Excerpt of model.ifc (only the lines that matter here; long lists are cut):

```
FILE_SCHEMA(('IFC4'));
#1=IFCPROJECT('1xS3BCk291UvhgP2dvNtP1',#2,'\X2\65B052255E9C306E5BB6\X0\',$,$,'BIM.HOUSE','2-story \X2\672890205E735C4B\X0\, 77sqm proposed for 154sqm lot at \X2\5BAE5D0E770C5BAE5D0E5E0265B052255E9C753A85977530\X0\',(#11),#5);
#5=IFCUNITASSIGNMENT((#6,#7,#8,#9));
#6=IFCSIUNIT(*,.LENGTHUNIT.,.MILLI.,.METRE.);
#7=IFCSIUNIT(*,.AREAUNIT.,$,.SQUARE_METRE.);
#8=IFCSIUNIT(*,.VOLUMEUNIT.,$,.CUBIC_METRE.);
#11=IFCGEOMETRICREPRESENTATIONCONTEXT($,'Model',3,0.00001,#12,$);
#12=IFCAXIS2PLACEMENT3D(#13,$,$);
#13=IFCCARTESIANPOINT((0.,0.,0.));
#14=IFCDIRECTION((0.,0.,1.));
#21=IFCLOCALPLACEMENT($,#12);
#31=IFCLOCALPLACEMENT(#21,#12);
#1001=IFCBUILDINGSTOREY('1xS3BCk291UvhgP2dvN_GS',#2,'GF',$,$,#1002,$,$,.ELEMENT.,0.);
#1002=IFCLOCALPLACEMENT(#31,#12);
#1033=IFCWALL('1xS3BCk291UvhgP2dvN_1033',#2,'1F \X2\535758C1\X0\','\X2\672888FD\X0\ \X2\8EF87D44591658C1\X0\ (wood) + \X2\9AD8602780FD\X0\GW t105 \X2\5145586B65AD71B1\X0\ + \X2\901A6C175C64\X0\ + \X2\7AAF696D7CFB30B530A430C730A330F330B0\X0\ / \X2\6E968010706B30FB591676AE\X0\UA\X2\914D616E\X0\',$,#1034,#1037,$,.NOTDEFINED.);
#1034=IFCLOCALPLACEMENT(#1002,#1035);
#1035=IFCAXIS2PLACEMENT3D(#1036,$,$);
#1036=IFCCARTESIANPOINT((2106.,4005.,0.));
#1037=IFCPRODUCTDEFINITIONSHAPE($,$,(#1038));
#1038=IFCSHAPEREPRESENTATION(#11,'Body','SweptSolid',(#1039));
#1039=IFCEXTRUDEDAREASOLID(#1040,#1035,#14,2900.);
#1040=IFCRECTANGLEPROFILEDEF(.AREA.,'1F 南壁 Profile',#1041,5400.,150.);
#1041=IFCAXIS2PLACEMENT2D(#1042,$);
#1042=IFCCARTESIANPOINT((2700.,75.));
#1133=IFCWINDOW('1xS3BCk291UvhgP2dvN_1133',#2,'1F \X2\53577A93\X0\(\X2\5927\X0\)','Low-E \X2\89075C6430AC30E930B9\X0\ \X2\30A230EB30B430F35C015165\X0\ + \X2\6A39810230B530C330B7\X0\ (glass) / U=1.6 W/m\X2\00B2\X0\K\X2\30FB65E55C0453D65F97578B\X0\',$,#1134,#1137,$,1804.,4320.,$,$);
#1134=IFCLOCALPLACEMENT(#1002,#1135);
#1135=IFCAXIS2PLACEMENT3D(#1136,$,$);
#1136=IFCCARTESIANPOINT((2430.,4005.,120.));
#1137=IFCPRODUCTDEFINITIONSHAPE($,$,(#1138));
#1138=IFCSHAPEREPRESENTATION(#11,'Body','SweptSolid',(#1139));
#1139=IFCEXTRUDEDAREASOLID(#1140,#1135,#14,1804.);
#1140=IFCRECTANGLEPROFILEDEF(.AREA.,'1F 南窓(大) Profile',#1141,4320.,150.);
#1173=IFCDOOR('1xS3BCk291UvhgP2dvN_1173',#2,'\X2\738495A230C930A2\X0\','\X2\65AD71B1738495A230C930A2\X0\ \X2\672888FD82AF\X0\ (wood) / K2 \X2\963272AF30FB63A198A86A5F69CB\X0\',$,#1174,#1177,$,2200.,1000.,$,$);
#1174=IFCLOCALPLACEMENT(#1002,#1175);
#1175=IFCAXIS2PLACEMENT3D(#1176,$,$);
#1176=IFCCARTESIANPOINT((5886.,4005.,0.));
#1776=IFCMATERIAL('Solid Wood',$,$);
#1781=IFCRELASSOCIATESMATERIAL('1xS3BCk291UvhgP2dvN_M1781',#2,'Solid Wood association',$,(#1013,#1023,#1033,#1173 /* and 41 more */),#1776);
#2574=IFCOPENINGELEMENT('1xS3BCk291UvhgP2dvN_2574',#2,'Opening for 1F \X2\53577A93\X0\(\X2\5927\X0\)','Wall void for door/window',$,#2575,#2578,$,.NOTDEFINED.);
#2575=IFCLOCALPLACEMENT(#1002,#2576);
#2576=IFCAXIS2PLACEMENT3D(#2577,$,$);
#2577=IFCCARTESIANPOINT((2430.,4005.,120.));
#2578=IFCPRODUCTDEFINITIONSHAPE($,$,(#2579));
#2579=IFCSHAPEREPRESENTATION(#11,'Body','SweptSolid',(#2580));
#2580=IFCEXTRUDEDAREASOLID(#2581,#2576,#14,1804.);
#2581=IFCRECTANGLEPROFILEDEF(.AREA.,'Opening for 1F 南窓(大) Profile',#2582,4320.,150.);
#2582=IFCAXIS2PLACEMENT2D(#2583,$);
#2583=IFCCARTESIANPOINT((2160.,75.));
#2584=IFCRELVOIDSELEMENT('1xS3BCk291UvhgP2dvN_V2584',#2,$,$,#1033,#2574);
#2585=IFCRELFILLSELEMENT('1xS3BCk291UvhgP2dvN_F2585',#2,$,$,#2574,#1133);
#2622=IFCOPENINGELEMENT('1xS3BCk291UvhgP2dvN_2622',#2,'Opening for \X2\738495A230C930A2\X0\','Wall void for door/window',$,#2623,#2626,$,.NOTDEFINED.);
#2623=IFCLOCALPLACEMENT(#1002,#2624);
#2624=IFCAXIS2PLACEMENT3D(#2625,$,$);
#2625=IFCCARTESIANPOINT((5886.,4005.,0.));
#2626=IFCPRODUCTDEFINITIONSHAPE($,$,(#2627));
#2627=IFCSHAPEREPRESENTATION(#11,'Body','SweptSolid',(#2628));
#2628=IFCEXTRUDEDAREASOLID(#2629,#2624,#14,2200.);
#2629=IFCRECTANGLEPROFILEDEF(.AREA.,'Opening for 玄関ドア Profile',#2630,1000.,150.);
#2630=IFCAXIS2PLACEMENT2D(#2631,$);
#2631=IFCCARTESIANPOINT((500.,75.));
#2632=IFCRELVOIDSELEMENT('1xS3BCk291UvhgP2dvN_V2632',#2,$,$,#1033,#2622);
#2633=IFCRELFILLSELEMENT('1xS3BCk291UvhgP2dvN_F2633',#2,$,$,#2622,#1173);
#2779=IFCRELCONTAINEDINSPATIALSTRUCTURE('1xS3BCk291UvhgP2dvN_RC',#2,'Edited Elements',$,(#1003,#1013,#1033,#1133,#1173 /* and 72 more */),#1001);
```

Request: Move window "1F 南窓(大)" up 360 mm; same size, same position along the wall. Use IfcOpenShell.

```python
import numpy as np
import ifcopenshell
import ifcopenshell.api.geometry
import ifcopenshell.util.placement
import ifcopenshell.util.unit

model = ifcopenshell.open("model.ifc")
unit_scale = ifcopenshell.util.unit.calculate_unit_scale(model)

window = model.by_guid("1xS3BCk291UvhgP2dvN_1133")
opening = window.FillsVoids[0].RelatingOpeningElement
dz = 0.36 / unit_scale

shift = np.array([0.0, 0.0, dz])
# The window is not placed relative to its opening, so move both.
for product in (opening, window):
    matrix = ifcopenshell.util.placement.get_local_placement(product.ObjectPlacement)
    matrix[:3, 3] += shift
    ifcopenshell.api.geometry.edit_object_placement(model, product=product, matrix=matrix, is_si=False)

print(f"moved by {dz * unit_scale:+.3f} m")

model.write("model_v2.ifc")
```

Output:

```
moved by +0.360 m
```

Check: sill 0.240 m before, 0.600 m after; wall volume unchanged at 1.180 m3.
